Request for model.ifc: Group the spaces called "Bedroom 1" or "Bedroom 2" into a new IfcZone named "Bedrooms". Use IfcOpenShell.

First a look at what the model holds.

```python
import ifcopenshell

model = ifcopenshell.open("model.ifc")
print(model.schema)
seen = {}
for space in model.by_type("IfcSpace"):
    seen[space.LongName] = seen.get(space.LongName, 0) + 1
for name, count in sorted(seen.items(), key=str):
    print(count, "x", name)
print("zones:", [z.Name for z in model.by_type("IfcZone")][:20])
```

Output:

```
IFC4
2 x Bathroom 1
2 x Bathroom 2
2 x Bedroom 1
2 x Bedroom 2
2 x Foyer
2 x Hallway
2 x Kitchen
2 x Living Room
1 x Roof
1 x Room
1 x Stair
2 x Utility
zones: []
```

```python
import ifcopenshell
import ifcopenshell.api.group
import ifcopenshell.api.root

model = ifcopenshell.open("model.ifc")

names = {"Bedroom 1", "Bedroom 2"}
spaces = [s for s in model.by_type("IfcSpace") if s.LongName in names]

zone = ifcopenshell.api.root.create_entity(model, ifc_class="IfcZone", name="Bedrooms")
ifcopenshell.api.group.assign_group(model, products=spaces, group=zone)
print(len(spaces), "spaces in", zone.Name)

model.write("model-out.ifc")
```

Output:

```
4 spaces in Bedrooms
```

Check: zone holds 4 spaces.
